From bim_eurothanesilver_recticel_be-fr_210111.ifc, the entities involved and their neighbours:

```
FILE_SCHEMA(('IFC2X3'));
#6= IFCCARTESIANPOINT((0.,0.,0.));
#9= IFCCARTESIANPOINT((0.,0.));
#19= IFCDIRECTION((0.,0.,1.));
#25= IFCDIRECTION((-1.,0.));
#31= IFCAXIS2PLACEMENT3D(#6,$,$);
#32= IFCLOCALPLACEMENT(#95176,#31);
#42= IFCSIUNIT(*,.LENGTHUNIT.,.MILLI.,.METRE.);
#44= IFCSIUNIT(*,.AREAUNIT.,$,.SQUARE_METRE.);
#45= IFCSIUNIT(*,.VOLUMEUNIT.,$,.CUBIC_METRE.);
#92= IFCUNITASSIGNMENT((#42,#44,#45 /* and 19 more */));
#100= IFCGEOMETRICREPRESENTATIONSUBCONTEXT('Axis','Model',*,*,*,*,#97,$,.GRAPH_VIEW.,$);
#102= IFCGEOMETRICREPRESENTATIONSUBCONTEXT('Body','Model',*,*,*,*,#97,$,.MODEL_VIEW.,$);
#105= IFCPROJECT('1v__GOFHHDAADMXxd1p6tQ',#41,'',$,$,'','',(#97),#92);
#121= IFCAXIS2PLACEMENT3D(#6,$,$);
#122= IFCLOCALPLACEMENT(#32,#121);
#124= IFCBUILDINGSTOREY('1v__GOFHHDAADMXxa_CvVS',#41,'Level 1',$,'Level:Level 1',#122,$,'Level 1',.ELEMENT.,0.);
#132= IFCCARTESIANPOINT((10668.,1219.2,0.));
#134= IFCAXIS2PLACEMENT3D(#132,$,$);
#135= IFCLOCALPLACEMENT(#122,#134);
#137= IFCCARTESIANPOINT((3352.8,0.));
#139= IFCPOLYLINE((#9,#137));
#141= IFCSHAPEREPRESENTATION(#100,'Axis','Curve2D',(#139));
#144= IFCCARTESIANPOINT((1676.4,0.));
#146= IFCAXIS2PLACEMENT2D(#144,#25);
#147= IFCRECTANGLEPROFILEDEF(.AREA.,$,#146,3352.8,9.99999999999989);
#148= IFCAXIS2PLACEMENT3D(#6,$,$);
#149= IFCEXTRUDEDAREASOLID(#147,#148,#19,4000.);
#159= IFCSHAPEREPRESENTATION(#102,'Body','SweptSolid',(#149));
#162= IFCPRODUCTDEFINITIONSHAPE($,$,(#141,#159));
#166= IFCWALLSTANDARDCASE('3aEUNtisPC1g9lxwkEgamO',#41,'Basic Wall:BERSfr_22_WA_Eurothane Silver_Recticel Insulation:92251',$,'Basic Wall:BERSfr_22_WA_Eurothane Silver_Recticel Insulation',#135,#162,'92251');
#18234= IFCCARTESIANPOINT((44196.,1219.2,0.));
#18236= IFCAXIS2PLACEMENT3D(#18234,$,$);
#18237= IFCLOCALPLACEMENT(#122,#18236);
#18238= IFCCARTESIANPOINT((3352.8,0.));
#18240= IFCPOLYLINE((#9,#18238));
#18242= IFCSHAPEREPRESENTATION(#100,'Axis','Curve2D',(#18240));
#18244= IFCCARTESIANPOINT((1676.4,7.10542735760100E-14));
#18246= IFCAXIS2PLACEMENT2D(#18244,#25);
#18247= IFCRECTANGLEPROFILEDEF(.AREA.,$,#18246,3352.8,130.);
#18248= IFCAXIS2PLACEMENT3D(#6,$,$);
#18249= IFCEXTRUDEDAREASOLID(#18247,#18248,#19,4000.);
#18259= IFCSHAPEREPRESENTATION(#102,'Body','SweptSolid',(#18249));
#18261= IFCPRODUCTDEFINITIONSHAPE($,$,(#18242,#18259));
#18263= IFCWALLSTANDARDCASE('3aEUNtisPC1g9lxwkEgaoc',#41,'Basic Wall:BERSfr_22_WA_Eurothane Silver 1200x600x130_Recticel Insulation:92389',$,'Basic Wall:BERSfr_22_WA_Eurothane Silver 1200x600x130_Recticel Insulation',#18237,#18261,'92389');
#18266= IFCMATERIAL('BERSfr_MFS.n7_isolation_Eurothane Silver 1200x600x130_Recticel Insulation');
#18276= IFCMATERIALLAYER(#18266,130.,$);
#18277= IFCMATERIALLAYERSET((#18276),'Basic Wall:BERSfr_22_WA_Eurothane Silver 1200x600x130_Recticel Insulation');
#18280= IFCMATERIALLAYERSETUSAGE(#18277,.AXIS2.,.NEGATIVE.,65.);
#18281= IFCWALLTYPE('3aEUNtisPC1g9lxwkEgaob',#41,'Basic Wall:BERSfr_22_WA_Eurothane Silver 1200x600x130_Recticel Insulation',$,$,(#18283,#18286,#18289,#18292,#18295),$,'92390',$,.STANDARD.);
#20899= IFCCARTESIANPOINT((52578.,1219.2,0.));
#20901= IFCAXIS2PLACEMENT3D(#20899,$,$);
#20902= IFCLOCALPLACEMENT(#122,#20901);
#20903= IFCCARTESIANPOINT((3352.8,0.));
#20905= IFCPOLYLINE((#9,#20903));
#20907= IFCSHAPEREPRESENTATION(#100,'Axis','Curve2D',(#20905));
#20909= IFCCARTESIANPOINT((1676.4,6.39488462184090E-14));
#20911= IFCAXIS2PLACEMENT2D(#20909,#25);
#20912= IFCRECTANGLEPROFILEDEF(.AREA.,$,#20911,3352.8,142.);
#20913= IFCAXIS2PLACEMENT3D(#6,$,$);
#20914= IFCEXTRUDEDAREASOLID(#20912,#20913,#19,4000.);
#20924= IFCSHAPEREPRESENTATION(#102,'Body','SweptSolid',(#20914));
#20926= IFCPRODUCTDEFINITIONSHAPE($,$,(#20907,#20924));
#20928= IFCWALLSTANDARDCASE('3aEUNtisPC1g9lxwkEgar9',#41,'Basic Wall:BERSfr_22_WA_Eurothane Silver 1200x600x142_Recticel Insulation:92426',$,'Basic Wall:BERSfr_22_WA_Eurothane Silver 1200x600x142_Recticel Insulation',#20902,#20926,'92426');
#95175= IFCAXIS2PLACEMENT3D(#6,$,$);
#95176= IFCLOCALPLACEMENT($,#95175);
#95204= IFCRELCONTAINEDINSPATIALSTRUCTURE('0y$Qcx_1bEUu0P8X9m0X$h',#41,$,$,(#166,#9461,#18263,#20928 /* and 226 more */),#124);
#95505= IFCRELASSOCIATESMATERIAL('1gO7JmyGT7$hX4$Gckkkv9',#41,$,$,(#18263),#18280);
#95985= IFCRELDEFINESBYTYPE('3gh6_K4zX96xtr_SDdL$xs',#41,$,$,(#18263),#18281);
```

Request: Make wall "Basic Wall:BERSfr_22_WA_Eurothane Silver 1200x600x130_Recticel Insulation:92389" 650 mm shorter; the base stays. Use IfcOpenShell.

```python
import ifcopenshell
import ifcopenshell.geom
import ifcopenshell.util.representation
import ifcopenshell.util.shape
import ifcopenshell.util.unit

model = ifcopenshell.open("bim_eurothanesilver_recticel_be-fr_210111.ifc")
unit_scale = ifcopenshell.util.unit.calculate_unit_scale(model)
settings = ifcopenshell.geom.settings()


def volume(element):
    """Net volume in cubic metres, openings subtracted."""
    shape = ifcopenshell.geom.create_shape(settings, element)
    return ifcopenshell.util.shape.get_volume(shape.geometry)


wall = model.by_guid("3aEUNtisPC1g9lxwkEgaoc")
before = volume(wall)

body = ifcopenshell.util.representation.get_representation(wall, "Model", "Body")
solid = body.Items[0]
old_height = solid.Depth
solid.Depth -= 0.65 / unit_scale
after = volume(wall)

print(f"height {old_height:g} -> {solid.Depth:g}, volume {before:.3f} -> {after:.3f} m3")

model.write("bim_eurothanesilver_recticel_be-fr_210111_updated.ifc")
```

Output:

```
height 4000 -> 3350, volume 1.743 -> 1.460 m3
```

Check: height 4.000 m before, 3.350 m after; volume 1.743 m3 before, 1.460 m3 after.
